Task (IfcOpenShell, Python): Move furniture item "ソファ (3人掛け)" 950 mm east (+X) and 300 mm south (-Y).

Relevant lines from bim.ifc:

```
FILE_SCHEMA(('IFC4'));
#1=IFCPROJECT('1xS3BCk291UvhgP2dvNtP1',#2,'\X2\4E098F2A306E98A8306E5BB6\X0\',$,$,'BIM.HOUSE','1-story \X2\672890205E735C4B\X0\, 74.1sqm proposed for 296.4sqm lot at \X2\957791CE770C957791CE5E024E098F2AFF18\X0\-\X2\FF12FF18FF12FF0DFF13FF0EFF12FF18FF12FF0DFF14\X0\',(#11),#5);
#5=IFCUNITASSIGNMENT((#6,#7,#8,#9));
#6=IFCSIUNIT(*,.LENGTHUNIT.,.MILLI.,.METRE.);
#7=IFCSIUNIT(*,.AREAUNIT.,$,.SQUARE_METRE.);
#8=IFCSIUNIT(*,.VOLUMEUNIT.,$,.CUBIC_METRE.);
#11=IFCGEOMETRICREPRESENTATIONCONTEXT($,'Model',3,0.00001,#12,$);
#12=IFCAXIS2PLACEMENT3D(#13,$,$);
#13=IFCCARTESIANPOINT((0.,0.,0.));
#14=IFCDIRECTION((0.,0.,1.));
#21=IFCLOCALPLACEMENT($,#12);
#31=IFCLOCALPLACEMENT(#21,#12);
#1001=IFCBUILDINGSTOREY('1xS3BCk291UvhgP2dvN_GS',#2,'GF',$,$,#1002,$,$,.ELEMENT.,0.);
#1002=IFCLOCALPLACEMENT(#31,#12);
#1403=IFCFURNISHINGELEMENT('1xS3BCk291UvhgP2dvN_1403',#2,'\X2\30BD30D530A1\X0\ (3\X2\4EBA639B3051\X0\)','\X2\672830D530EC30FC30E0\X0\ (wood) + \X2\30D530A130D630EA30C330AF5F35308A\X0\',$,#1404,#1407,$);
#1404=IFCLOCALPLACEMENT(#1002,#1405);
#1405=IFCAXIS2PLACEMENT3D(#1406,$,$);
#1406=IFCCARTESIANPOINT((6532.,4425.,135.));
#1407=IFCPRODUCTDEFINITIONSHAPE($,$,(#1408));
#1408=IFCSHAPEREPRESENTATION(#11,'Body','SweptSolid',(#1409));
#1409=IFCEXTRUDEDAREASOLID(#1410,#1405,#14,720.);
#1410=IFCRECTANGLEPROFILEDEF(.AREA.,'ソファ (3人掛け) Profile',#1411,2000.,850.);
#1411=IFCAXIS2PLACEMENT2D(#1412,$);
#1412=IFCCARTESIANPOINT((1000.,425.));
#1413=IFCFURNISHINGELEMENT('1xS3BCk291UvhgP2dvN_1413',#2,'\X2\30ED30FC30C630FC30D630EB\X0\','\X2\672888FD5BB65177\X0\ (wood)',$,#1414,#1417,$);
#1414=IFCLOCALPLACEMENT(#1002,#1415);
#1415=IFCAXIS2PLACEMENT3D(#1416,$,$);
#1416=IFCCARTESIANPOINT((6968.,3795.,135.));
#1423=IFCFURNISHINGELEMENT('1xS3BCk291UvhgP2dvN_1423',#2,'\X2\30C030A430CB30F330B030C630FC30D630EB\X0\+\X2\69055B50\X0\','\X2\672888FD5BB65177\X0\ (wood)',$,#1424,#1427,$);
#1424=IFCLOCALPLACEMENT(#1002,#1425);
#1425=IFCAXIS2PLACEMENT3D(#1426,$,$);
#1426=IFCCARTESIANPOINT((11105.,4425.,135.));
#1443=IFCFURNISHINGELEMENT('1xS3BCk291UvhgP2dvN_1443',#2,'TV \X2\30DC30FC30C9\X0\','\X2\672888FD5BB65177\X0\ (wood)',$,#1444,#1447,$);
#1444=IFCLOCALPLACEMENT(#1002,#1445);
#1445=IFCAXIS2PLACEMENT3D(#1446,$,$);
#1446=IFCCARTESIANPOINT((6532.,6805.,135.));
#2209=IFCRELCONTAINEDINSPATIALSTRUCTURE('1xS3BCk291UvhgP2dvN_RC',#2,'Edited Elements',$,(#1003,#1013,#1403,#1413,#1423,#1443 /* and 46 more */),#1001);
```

```python
import ifcopenshell
import ifcopenshell.api.geometry
import ifcopenshell.util.placement
import ifcopenshell.util.unit

model = ifcopenshell.open("bim.ifc")
unit_scale = ifcopenshell.util.unit.calculate_unit_scale(model)

item = model.by_id(1403)
matrix = ifcopenshell.util.placement.get_local_placement(item.ObjectPlacement)
matrix[0, 3] += 0.95 / unit_scale
matrix[1, 3] -= 0.3 / unit_scale
ifcopenshell.api.geometry.edit_object_placement(model, product=item, matrix=matrix, is_si=False)

print(ifcopenshell.util.placement.get_local_placement(item.ObjectPlacement).round(3) + 0.0)

model.write("bim-out.ifc")
```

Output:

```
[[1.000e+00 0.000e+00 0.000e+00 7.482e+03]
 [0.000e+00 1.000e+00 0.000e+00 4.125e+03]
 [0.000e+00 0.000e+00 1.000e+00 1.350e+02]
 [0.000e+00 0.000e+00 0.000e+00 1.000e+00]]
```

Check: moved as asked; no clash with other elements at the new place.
